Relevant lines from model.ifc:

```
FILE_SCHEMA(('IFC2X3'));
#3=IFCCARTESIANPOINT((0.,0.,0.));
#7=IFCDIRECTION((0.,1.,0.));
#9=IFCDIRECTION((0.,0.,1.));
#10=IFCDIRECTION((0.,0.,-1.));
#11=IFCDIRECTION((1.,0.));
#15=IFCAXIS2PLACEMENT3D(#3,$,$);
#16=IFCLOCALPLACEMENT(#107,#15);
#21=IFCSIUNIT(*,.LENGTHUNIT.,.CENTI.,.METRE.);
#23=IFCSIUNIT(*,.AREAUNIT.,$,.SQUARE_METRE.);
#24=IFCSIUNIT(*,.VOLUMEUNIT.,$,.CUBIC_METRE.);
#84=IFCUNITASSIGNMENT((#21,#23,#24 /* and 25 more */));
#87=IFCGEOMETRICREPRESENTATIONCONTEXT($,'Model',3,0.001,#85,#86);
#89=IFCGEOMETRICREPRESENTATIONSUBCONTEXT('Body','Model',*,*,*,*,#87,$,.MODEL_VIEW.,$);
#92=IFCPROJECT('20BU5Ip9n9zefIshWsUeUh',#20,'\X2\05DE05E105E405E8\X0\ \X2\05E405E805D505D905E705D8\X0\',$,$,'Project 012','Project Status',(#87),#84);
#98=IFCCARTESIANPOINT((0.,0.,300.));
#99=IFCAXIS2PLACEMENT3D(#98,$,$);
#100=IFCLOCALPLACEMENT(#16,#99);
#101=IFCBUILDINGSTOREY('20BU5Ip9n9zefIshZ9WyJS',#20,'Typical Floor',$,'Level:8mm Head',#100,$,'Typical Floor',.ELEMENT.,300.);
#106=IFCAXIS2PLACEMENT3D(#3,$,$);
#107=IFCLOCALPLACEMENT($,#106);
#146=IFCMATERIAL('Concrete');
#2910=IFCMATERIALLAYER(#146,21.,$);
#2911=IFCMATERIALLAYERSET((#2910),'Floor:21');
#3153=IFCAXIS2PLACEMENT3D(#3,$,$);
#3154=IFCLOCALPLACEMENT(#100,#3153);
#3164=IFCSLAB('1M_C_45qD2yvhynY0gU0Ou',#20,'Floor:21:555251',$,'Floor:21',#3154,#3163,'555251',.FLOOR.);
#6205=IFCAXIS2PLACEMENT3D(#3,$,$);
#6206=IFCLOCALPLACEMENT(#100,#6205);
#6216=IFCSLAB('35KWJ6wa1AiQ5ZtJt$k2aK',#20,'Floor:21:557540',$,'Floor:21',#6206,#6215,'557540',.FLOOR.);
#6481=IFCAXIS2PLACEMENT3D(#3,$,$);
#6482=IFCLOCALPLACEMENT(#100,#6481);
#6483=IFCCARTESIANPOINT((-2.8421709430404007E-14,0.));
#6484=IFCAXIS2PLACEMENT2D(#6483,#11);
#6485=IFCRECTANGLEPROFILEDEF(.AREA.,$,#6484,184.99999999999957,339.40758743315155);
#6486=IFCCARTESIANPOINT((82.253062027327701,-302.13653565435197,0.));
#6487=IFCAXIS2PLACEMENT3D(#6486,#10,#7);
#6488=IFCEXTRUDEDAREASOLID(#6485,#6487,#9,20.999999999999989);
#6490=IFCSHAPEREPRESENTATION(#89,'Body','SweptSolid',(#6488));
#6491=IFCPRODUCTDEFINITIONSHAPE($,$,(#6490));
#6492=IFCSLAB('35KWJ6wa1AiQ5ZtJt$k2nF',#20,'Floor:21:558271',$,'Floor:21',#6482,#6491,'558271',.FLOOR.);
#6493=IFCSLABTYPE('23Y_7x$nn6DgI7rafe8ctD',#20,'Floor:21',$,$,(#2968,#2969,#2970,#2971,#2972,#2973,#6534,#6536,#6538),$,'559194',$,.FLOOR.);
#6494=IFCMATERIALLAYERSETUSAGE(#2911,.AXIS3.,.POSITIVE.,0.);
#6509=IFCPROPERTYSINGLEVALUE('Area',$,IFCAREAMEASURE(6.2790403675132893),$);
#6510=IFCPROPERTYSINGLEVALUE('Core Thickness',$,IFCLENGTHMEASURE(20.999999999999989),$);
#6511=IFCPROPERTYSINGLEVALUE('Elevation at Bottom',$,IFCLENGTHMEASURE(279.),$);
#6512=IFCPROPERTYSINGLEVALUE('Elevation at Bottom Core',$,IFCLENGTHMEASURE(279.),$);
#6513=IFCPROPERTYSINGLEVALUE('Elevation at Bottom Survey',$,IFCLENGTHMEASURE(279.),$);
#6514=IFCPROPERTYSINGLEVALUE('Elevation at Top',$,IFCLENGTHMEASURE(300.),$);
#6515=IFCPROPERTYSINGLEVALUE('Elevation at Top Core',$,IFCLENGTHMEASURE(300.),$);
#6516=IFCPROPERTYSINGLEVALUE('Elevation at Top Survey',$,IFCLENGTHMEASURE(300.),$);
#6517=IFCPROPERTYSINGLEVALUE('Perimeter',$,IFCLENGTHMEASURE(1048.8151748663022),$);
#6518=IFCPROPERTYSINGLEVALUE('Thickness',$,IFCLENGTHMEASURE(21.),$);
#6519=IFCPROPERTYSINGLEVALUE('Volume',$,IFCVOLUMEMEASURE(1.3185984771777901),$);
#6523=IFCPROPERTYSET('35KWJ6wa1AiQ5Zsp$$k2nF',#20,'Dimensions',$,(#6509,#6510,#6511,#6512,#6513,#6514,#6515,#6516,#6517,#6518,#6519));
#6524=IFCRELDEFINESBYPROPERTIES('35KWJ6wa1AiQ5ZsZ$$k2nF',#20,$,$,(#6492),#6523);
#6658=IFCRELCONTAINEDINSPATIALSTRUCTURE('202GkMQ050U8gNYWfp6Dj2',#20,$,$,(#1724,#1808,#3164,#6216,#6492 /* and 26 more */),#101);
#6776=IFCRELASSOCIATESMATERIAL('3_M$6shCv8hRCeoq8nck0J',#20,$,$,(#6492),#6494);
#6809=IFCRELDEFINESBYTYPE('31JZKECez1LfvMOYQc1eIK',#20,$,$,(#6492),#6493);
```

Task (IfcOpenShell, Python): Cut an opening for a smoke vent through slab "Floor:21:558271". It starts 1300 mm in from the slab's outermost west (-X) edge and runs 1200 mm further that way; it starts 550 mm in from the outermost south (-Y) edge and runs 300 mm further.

```python
import numpy as np
import ifcopenshell
import ifcopenshell.api.feature
import ifcopenshell.api.geometry
import ifcopenshell.api.pset
import ifcopenshell.api.root
import ifcopenshell.geom
import ifcopenshell.util.element
import ifcopenshell.util.placement
import ifcopenshell.util.representation
import ifcopenshell.util.shape
import ifcopenshell.util.unit

model = ifcopenshell.open("model.ifc")
unit_scale = ifcopenshell.util.unit.calculate_unit_scale(model)
area_scale = ifcopenshell.util.unit.calculate_unit_scale(model, "AREAUNIT")
volume_scale = ifcopenshell.util.unit.calculate_unit_scale(model, "VOLUMEUNIT")
settings = ifcopenshell.geom.settings()


def volume(element):
    """Net volume in cubic metres, openings subtracted."""
    shape = ifcopenshell.geom.create_shape(settings, element)
    return ifcopenshell.util.shape.get_volume(shape.geometry)


slab = model.by_id(6492)
before = volume(slab)

# Extent in the slab's own axes, in metres. The edges named are its -X and -Y sides.
slab_shape = ifcopenshell.geom.create_shape(settings, slab)
vertices = ifcopenshell.util.shape.get_vertices(slab_shape.geometry)
x_min, y_min, bottom = vertices.min(axis=0)
top = vertices[:, 2].max()

opening = ifcopenshell.api.root.create_entity(model, ifc_class="IfcOpeningElement", name="Smoke vent opening")
context = ifcopenshell.util.representation.get_context(model, "Model", "Body", "MODEL_VIEW")
width, depth = 1.2, 0.3
outline = [(0.0, 0.0), (width, 0.0), (width, depth), (0.0, depth), (0.0, 0.0)]
# Overshoot both faces by 50 mm so the cut is clean.
shape = ifcopenshell.api.geometry.add_slab_representation(
    model, context=context, depth=top - bottom + 0.1, polyline=outline
)
ifcopenshell.api.geometry.assign_representation(model, product=opening, representation=shape)

matrix = ifcopenshell.util.placement.get_local_placement(slab.ObjectPlacement)
matrix[:, 3] = matrix @ np.append(np.array([x_min + 1.3, y_min + 0.55, bottom - 0.05]) / unit_scale, 1.0)
ifcopenshell.api.geometry.edit_object_placement(model, product=opening, matrix=matrix, is_si=False)
ifcopenshell.api.feature.add_feature(model, feature=opening, element=slab)

after = volume(slab)

# Update the slab's stored quantities.
pset = model.by_id(ifcopenshell.util.element.get_pset(slab, "Dimensions", should_inherit=False)["id"])
ifcopenshell.api.pset.edit_pset(model, pset=pset, properties={
    "Area": model.create_entity("IfcAreaMeasure", after / (top - bottom) / area_scale),
    "Volume": model.create_entity("IfcVolumeMeasure", after / volume_scale),
})

print(f"slab volume {before:.3f} -> {after:.3f} m3")

model.write("model_updated.ifc")
```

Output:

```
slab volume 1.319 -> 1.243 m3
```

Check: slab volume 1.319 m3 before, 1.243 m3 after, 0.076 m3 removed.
